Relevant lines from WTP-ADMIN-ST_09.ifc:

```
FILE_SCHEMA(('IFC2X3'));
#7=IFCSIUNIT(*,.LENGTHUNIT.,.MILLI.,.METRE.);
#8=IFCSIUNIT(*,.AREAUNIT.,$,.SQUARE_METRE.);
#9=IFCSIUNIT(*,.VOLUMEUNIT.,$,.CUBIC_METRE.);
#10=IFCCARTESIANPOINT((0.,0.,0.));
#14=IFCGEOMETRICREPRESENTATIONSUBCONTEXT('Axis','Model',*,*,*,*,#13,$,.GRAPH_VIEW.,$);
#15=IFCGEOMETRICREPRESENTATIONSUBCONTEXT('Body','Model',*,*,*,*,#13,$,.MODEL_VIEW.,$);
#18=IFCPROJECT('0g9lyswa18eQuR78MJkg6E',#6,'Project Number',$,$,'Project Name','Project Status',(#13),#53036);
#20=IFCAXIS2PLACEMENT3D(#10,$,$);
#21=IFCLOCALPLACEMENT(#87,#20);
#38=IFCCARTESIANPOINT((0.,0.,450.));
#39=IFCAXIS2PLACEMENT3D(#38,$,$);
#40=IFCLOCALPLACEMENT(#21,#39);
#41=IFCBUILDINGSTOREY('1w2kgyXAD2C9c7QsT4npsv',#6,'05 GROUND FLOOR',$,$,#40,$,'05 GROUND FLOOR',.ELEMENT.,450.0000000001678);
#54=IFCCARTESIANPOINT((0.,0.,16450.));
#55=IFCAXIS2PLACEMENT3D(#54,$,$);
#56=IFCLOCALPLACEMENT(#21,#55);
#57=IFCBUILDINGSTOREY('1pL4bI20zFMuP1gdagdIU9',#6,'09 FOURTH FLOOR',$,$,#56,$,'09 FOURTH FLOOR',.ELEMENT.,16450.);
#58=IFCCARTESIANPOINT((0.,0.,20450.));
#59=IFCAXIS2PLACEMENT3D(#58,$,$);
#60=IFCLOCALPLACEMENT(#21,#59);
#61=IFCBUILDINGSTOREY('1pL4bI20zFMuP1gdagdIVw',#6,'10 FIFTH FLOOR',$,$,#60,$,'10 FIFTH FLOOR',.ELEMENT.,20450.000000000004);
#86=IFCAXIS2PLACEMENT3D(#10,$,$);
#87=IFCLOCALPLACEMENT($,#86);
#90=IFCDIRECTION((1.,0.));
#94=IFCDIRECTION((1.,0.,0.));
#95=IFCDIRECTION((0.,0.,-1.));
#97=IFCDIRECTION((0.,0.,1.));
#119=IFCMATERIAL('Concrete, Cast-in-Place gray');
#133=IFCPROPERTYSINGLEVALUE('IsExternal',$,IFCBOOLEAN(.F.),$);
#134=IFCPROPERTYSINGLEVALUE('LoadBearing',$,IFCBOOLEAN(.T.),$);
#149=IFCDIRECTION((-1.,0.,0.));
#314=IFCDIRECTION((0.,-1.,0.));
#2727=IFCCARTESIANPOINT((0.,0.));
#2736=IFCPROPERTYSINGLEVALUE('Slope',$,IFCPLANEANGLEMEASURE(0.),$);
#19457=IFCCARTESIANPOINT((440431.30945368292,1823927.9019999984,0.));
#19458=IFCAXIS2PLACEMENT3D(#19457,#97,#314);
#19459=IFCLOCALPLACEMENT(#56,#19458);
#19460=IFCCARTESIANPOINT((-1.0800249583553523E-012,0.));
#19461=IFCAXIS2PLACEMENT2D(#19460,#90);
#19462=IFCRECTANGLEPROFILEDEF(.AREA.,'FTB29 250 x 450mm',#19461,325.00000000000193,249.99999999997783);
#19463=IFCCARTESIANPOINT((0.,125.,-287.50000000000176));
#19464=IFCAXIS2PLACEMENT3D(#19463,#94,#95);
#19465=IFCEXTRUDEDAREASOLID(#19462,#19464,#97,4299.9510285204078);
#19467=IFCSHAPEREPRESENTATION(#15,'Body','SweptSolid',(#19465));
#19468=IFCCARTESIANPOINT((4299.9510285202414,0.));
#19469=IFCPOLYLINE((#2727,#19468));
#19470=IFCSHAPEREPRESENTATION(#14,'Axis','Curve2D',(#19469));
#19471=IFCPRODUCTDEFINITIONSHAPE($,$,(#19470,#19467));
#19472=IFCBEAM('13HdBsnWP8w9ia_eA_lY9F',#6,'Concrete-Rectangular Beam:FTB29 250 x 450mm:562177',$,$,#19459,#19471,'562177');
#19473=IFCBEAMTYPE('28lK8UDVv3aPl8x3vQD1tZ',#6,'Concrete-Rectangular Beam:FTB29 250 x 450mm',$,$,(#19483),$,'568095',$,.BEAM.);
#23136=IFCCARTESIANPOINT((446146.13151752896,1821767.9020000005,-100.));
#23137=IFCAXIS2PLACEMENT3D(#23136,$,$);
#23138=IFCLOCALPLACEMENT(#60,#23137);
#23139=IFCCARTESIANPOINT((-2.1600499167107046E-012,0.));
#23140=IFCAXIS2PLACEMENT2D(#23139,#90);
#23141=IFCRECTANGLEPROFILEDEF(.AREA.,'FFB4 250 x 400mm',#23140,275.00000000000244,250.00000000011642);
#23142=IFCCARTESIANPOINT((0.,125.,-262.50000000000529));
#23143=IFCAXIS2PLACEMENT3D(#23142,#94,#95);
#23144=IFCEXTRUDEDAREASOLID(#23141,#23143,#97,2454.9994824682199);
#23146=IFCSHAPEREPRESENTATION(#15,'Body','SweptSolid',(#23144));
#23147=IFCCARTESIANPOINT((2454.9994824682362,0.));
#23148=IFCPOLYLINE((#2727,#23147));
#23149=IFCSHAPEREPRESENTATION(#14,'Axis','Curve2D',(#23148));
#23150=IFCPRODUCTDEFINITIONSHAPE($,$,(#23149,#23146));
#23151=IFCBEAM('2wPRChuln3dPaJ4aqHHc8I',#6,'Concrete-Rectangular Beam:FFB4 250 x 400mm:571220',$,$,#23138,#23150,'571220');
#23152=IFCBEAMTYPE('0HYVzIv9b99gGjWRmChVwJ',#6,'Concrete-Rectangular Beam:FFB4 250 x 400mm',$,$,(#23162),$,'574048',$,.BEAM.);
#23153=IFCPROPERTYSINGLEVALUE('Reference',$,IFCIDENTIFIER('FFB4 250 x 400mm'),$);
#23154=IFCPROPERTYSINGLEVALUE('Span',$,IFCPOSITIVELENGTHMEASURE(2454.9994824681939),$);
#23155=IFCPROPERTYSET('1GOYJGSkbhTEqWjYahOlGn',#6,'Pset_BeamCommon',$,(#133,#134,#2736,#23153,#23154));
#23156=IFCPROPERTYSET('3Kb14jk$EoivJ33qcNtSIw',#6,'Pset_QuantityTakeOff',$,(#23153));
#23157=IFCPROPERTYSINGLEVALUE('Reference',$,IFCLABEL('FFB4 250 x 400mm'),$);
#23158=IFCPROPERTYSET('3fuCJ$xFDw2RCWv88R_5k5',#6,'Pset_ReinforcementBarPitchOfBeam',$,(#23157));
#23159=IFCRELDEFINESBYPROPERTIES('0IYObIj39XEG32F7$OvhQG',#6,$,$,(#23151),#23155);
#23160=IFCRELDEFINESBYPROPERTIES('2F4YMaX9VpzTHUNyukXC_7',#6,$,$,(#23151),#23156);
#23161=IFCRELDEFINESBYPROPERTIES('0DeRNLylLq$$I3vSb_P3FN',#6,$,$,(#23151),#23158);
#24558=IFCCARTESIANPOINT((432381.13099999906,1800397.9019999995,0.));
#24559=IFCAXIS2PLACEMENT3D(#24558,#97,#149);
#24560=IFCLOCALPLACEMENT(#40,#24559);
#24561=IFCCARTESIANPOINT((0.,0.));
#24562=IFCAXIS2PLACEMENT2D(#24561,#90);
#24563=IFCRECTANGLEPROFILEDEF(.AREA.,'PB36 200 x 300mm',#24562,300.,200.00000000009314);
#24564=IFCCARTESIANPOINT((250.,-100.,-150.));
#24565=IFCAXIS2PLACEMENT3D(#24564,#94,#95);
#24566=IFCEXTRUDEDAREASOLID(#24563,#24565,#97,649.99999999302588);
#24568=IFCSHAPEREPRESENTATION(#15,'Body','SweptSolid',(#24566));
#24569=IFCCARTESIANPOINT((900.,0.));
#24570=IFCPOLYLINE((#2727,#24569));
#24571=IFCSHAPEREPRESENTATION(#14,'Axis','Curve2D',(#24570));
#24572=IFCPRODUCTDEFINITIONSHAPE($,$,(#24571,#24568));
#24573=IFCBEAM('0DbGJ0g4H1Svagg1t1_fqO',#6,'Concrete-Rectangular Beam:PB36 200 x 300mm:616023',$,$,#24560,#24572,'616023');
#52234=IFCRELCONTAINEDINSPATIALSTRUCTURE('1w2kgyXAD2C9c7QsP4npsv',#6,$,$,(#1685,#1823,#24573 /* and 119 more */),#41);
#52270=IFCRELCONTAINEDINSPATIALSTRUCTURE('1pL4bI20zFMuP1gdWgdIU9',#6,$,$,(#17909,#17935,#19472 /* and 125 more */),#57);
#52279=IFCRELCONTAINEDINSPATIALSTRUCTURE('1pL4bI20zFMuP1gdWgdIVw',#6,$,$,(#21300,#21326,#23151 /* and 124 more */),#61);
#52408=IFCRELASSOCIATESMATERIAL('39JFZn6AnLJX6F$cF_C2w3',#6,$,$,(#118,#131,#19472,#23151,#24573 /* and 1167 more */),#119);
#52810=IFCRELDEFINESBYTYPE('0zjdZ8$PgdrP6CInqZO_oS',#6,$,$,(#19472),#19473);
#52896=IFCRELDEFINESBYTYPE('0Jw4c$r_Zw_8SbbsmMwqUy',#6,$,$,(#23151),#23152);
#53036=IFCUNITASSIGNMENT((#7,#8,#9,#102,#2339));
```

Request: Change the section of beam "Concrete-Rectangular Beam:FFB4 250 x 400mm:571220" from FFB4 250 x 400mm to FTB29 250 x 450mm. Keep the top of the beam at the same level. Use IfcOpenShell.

```python
import ifcopenshell
import ifcopenshell.api.pset
import ifcopenshell.api.type
import ifcopenshell.util.element
import ifcopenshell.util.representation

model = ifcopenshell.open("WTP-ADMIN-ST_09.ifc")

member = model.by_guid("2wPRChuln3dPaJ4aqHHc8I")
source = next(p for p in model.by_type("IfcRectangleProfileDef") if p.ProfileName == "FTB29 250 x 450mm")

body = ifcopenshell.util.representation.get_representation(member, "Model", "Body")
solid = body.Items[0]
old_profile = solid.SweptArea

# Copy the section's sizes but keep this member's own profile position.
profile = ifcopenshell.util.element.copy(model, source)
# Profiles are centred, so shift by half the change in depth to hold the top.
shift = (old_profile.XDim - profile.XDim) / 2
x, y = old_profile.Position.Location.Coordinates
up = (-1.0, 0.0)  # upwards, in the solid's own plane
location = model.createIfcCartesianPoint((x + up[0] * shift, y + up[1] * shift))
profile.Position = model.createIfcAxis2Placement2D(location, old_profile.Position.RefDirection)
solid.SweptArea = profile
if not model.get_total_inverses(old_profile):
    ifcopenshell.util.element.remove_deep2(model, old_profile)

new_type = model.by_guid("28lK8UDVv3aPl8x3vQD1tZ")
ifcopenshell.api.type.assign_type(
    model, related_objects=[member], relating_type=new_type, should_map_representations=False
)
member.Name = member.Name.replace("FFB4 250 x 400mm", "FTB29 250 x 450mm")
pset = model.by_id(ifcopenshell.util.element.get_pset(member, "Pset_BeamCommon", should_inherit=False)["id"])
ifcopenshell.api.pset.edit_pset(model, pset=pset, properties={"Reference": "FTB29 250 x 450mm"})
pset = model.by_id(ifcopenshell.util.element.get_pset(member, "Pset_QuantityTakeOff", should_inherit=False)["id"])
ifcopenshell.api.pset.edit_pset(model, pset=pset, properties={"Reference": "FTB29 250 x 450mm"})
pset = model.by_id(ifcopenshell.util.element.get_pset(member, "Pset_ReinforcementBarPitchOfBeam", should_inherit=False)["id"])
ifcopenshell.api.pset.edit_pset(model, pset=pset, properties={"Reference": "FTB29 250 x 450mm"})

print(solid.SweptArea)

model.write("WTP-ADMIN-ST_09_rev.ifc")
```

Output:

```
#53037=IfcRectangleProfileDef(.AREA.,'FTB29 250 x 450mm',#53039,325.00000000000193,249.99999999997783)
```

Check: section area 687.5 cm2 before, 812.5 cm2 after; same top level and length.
